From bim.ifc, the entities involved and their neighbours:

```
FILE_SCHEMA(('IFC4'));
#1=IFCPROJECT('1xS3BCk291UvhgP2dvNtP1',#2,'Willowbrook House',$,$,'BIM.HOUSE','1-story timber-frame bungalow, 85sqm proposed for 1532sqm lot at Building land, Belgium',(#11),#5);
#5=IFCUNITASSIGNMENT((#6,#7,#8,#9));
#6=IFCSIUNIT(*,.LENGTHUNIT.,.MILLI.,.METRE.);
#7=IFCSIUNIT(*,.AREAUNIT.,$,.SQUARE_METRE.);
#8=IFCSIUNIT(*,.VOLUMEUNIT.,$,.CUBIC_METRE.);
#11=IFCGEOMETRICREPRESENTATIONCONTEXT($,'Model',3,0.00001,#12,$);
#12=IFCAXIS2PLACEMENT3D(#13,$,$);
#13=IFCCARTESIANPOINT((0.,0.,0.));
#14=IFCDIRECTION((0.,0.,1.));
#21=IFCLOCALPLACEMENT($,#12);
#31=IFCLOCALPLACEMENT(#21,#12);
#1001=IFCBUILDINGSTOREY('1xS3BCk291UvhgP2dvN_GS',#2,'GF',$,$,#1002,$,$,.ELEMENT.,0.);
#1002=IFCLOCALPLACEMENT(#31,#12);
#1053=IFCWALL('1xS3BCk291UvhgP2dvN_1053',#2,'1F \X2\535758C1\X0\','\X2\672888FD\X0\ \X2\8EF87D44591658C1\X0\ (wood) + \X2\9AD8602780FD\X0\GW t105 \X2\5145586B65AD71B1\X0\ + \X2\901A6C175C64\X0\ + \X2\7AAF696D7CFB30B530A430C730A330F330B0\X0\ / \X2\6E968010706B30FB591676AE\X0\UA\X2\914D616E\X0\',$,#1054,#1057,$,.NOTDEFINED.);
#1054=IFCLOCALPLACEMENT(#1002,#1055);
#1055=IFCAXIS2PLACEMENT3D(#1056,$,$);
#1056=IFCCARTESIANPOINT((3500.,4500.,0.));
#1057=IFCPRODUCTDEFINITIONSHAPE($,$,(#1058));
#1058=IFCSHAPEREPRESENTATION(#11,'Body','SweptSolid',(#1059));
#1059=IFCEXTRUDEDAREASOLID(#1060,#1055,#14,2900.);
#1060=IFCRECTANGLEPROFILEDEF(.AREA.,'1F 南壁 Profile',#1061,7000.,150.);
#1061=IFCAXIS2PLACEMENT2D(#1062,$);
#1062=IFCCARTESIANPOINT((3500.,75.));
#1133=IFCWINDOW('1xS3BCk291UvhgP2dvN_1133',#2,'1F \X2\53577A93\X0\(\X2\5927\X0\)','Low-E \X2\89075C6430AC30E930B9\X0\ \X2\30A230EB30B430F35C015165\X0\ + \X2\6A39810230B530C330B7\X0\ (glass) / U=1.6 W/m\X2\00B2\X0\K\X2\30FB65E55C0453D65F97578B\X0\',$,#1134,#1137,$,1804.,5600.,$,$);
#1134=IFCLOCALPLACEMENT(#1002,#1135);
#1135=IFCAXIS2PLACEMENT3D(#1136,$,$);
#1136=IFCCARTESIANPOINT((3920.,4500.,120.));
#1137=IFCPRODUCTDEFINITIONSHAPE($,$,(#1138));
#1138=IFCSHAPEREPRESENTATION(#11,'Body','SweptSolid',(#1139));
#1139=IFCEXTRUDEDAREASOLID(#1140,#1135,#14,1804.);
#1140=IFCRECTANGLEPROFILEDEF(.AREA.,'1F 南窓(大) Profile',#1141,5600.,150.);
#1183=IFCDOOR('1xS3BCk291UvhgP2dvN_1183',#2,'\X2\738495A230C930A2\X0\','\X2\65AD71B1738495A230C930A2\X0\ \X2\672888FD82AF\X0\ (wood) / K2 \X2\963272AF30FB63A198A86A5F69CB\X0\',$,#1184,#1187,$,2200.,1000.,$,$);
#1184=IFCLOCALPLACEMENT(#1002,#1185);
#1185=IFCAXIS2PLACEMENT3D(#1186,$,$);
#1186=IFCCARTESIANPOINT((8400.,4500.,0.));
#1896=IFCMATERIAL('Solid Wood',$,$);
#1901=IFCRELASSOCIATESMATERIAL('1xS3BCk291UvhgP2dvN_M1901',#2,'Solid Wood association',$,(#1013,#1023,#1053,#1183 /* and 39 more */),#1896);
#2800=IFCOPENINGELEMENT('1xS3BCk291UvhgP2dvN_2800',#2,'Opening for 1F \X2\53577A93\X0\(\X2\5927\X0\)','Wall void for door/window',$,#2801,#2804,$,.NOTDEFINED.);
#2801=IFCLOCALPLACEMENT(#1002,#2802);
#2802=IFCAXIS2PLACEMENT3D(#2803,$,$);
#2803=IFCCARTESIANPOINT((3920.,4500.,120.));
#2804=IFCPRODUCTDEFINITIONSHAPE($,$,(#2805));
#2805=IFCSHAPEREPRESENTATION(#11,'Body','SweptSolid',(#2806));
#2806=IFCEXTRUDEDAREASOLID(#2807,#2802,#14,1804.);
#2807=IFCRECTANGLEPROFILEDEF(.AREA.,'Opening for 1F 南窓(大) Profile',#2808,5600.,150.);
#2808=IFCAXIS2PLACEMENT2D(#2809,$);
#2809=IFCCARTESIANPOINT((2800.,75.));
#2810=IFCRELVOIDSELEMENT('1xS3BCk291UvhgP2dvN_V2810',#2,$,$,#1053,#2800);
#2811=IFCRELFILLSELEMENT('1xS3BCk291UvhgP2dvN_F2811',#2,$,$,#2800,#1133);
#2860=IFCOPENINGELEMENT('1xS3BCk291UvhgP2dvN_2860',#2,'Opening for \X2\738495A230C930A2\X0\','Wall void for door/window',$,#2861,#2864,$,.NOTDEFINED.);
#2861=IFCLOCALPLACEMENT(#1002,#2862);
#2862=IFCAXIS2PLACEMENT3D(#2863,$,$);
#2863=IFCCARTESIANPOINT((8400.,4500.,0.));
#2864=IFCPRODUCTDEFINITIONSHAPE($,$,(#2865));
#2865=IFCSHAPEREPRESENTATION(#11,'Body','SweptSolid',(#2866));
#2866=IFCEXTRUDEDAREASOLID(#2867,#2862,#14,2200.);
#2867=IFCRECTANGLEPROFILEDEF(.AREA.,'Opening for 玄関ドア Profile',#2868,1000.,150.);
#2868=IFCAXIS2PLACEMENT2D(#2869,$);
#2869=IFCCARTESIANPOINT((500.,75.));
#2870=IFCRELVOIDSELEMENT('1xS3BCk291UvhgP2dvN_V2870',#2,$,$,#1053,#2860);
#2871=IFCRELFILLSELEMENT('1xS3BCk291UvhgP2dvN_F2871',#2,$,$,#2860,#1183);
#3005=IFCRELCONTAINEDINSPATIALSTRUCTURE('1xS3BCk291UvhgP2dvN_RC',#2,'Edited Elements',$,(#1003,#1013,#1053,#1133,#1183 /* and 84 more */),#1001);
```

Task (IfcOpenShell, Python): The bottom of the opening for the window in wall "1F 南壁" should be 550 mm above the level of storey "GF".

```python
import numpy as np
import ifcopenshell
import ifcopenshell.api.geometry
import ifcopenshell.geom
import ifcopenshell.util.element
import ifcopenshell.util.placement
import ifcopenshell.util.shape
import ifcopenshell.util.unit

model = ifcopenshell.open("bim.ifc")
unit_scale = ifcopenshell.util.unit.calculate_unit_scale(model)

window = model.by_guid("1xS3BCk291UvhgP2dvN_1133")
opening = window.FillsVoids[0].RelatingOpeningElement
storey = ifcopenshell.util.element.get_container(window, ifc_class="IfcBuildingStorey")
level = ifcopenshell.util.placement.get_local_placement(storey.ObjectPlacement)[2, 3]

# The opening's origin need not be at the sill, so measure its lowest point.
shape = ifcopenshell.geom.create_shape(ifcopenshell.geom.settings(), opening)
bottom = ifcopenshell.util.shape.get_shape_bottom_elevation(shape, shape.geometry) / unit_scale
dz = level + 0.55 / unit_scale - bottom

shift = np.array([0.0, 0.0, dz])
# The window is not placed relative to its opening, so move both.
for product in (opening, window):
    matrix = ifcopenshell.util.placement.get_local_placement(product.ObjectPlacement)
    matrix[:3, 3] += shift
    ifcopenshell.api.geometry.edit_object_placement(model, product=product, matrix=matrix, is_si=False)

print(f"moved by {dz * unit_scale:+.3f} m")

model.write("bim_rev.ifc")
```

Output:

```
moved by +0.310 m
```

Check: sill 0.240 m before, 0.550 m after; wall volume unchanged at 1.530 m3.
